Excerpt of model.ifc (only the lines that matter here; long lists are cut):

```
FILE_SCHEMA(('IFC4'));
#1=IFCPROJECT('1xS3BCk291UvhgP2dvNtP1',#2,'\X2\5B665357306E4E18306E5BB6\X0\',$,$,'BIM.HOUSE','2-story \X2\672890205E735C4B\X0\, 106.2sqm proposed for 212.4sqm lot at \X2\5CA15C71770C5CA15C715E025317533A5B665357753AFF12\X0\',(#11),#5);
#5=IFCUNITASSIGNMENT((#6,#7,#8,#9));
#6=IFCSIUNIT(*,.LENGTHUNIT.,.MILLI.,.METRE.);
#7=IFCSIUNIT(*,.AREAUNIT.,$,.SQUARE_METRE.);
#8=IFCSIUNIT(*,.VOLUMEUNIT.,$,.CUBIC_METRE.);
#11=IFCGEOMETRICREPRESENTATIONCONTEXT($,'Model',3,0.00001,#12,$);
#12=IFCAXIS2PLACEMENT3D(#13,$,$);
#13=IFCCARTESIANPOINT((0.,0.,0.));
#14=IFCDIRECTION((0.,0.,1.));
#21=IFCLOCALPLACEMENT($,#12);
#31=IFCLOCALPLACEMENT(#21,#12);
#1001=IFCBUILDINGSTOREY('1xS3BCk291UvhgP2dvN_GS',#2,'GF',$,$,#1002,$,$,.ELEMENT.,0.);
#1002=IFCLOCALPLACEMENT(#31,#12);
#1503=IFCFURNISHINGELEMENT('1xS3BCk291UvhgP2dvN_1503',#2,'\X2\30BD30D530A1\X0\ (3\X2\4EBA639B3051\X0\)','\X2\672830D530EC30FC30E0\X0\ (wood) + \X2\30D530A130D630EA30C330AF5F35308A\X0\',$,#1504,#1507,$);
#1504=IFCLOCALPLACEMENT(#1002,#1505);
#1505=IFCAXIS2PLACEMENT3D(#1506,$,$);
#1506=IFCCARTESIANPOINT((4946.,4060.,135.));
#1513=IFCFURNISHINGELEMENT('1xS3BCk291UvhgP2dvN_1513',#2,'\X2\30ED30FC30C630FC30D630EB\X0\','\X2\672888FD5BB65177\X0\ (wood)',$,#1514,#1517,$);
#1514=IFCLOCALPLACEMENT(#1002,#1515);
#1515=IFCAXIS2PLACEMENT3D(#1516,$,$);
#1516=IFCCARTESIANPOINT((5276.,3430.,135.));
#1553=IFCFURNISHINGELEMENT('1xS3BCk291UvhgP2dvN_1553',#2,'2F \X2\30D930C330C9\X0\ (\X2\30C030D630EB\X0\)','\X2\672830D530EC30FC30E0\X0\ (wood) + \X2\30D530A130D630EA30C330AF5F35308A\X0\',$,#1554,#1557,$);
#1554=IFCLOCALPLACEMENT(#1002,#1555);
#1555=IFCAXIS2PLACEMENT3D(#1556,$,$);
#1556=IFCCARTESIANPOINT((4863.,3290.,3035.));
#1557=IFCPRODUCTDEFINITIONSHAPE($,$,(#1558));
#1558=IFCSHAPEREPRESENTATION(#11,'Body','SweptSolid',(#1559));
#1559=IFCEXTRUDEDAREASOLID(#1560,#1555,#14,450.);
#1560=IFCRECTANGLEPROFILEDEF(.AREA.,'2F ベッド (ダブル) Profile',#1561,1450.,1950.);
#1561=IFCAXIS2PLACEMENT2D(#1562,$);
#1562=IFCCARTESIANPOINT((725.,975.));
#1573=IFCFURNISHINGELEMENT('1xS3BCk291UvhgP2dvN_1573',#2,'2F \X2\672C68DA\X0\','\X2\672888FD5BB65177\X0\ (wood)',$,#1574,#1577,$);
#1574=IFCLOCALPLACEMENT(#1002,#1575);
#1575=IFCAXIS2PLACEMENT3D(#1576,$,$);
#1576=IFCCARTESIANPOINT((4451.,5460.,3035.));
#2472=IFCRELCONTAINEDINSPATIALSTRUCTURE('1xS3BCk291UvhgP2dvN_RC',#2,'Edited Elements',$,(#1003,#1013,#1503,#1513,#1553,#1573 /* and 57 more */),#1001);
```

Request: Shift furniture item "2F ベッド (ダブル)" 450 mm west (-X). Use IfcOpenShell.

```python
import ifcopenshell
import ifcopenshell.api.geometry
import ifcopenshell.util.placement
import ifcopenshell.util.unit

model = ifcopenshell.open("model.ifc")
unit_scale = ifcopenshell.util.unit.calculate_unit_scale(model)

item = model.by_id(1553)
matrix = ifcopenshell.util.placement.get_local_placement(item.ObjectPlacement)
matrix[0, 3] -= 0.45 / unit_scale
ifcopenshell.api.geometry.edit_object_placement(model, product=item, matrix=matrix, is_si=False)

print(ifcopenshell.util.placement.get_local_placement(item.ObjectPlacement).round(3) + 0.0)

model.write("model_updated.ifc")
```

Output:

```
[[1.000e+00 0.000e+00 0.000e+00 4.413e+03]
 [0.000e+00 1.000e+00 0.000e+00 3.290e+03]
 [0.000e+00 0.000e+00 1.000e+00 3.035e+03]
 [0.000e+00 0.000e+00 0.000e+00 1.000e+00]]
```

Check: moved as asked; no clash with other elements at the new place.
